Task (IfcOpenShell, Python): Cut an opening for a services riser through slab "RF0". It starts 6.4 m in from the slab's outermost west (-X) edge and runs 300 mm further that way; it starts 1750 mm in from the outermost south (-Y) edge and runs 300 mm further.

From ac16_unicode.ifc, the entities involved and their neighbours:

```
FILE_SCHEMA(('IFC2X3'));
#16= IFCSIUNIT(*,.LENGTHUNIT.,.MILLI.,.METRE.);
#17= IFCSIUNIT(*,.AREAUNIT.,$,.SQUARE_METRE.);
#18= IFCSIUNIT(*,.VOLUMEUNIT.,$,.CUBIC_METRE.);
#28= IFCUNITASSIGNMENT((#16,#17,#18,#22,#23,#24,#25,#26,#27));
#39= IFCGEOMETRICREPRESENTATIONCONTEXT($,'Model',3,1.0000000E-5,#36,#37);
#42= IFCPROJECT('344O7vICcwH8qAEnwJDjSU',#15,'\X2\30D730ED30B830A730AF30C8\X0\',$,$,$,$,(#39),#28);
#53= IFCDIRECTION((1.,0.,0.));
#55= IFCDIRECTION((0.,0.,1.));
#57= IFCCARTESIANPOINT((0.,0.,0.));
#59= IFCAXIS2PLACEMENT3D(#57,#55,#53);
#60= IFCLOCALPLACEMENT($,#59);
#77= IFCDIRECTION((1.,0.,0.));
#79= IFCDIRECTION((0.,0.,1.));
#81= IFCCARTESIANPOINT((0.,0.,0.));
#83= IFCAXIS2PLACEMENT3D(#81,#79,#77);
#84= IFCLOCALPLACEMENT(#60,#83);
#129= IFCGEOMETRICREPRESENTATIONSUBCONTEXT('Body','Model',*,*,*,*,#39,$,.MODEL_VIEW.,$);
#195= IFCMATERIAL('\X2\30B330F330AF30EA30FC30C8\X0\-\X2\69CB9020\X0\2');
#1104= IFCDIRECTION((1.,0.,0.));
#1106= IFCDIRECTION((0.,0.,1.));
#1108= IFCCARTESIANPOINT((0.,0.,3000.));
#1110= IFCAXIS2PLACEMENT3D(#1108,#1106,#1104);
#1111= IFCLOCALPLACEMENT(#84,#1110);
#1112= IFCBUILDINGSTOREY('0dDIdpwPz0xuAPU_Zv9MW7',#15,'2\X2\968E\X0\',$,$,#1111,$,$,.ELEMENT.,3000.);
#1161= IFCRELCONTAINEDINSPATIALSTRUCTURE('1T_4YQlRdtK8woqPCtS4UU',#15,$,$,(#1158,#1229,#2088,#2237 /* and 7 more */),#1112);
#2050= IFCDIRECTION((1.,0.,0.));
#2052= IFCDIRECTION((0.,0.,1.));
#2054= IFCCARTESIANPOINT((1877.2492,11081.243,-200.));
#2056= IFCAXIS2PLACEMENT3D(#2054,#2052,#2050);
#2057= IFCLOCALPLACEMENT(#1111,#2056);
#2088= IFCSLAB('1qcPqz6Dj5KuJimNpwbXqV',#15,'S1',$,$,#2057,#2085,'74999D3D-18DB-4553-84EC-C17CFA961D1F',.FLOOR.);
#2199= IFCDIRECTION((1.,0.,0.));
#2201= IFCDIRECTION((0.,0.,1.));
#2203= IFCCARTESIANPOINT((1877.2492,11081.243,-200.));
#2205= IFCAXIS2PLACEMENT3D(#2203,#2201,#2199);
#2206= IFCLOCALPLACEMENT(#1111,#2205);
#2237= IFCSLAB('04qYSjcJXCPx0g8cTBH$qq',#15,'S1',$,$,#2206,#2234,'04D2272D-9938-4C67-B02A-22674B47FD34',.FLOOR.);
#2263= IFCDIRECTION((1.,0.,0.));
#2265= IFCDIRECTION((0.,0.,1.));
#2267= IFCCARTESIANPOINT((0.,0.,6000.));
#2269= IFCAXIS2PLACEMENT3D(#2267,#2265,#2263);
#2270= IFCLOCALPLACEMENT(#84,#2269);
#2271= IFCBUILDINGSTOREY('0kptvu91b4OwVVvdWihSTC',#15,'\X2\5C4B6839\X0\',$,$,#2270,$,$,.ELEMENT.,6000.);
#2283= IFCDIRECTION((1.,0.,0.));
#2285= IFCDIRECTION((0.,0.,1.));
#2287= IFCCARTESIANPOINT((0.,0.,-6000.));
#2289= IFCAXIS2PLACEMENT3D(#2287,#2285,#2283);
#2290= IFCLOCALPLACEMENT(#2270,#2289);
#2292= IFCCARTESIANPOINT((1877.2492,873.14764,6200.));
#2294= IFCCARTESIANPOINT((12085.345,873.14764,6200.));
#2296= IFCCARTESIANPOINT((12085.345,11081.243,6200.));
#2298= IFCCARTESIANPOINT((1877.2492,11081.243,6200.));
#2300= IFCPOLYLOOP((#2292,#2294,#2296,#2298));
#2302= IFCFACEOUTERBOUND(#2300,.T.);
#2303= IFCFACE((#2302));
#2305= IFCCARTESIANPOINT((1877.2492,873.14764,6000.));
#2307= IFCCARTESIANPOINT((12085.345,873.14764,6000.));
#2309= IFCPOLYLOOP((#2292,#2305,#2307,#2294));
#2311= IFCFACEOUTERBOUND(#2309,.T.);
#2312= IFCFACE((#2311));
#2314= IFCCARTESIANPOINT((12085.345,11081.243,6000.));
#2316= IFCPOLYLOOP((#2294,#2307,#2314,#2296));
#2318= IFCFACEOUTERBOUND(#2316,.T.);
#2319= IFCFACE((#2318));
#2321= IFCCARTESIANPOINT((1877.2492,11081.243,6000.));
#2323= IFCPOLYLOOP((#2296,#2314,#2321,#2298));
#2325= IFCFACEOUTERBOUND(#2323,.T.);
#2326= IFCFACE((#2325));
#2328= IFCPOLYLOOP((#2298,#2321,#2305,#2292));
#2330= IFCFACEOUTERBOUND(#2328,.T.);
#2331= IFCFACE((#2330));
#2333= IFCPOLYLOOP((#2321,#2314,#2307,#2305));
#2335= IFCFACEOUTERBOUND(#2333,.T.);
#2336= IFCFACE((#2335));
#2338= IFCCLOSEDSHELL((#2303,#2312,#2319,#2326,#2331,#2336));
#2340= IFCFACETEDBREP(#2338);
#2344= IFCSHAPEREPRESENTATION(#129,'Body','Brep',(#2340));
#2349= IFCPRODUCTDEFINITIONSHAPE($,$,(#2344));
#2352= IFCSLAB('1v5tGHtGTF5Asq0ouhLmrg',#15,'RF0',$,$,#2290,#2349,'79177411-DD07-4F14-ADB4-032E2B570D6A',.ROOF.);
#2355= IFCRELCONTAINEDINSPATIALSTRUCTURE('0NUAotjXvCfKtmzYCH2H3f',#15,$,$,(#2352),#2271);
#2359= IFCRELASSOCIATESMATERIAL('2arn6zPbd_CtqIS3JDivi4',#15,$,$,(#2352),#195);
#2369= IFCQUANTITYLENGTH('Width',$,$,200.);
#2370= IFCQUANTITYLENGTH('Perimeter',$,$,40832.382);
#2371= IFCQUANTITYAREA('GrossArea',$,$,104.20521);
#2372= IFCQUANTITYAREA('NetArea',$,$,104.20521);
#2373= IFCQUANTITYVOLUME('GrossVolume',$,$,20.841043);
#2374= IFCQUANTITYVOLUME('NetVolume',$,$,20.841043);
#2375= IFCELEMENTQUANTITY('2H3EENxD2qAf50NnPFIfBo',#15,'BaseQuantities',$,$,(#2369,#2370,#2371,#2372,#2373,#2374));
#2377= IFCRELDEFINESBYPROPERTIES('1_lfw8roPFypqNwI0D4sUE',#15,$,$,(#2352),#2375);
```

```python
import numpy as np
import ifcopenshell
import ifcopenshell.api.feature
import ifcopenshell.api.geometry
import ifcopenshell.api.pset
import ifcopenshell.api.root
import ifcopenshell.geom
import ifcopenshell.util.element
import ifcopenshell.util.placement
import ifcopenshell.util.representation
import ifcopenshell.util.shape
import ifcopenshell.util.unit

model = ifcopenshell.open("ac16_unicode.ifc")
unit_scale = ifcopenshell.util.unit.calculate_unit_scale(model)
area_scale = ifcopenshell.util.unit.calculate_unit_scale(model, "AREAUNIT")
volume_scale = ifcopenshell.util.unit.calculate_unit_scale(model, "VOLUMEUNIT")
settings = ifcopenshell.geom.settings()


def volume(element):
    """Net volume in cubic metres, openings subtracted."""
    shape = ifcopenshell.geom.create_shape(settings, element)
    return ifcopenshell.util.shape.get_volume(shape.geometry)


slab = model.by_guid("1v5tGHtGTF5Asq0ouhLmrg")
before = volume(slab)

# Extent in the slab's own axes, in metres. The edges named are its -X and -Y sides.
slab_shape = ifcopenshell.geom.create_shape(settings, slab)
vertices = ifcopenshell.util.shape.get_vertices(slab_shape.geometry)
x_min, y_min, bottom = vertices.min(axis=0)
top = vertices[:, 2].max()

opening = ifcopenshell.api.root.create_entity(model, ifc_class="IfcOpeningElement", name="Services riser opening")
context = ifcopenshell.util.representation.get_context(model, "Model", "Body", "MODEL_VIEW")
width, depth = 0.3, 0.3
outline = [(0.0, 0.0), (width, 0.0), (width, depth), (0.0, depth), (0.0, 0.0)]
# Overshoot both faces by 50 mm so the cut is clean.
shape = ifcopenshell.api.geometry.add_slab_representation(
    model, context=context, depth=top - bottom + 0.1, polyline=outline
)
ifcopenshell.api.geometry.assign_representation(model, product=opening, representation=shape)

matrix = ifcopenshell.util.placement.get_local_placement(slab.ObjectPlacement)
matrix[:, 3] = matrix @ np.append(np.array([x_min + 6.4, y_min + 1.75, bottom - 0.05]) / unit_scale, 1.0)
ifcopenshell.api.geometry.edit_object_placement(model, product=opening, matrix=matrix, is_si=False)
ifcopenshell.api.feature.add_feature(model, feature=opening, element=slab)

after = volume(slab)

# Update the slab's stored quantities.
qto = model.by_id(ifcopenshell.util.element.get_pset(slab, "BaseQuantities", should_inherit=False)["id"])
ifcopenshell.api.pset.edit_qto(model, qto=qto, properties={
    "NetArea": after / (top - bottom) / area_scale,
    "NetVolume": after / volume_scale,
})

print(f"slab volume {before:.3f} -> {after:.3f} m3")

model.write("ac16_unicode_updated.ifc")
```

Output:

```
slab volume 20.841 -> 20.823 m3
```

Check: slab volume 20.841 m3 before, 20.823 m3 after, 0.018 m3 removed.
